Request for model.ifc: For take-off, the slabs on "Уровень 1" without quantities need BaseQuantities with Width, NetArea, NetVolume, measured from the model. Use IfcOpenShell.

First a look at what the model holds.

```python
import ifcopenshell
import ifcopenshell.util.element
import ifcopenshell.util.unit

model = ifcopenshell.open("model.ifc")
print(model.schema)
for unit_type in ("LENGTHUNIT", "AREAUNIT", "VOLUMEUNIT"):
    print(unit_type, ifcopenshell.util.unit.calculate_unit_scale(model, unit_type))
storey = next(s for s in model.by_type("IfcBuildingStorey") if s.Name == "Уровень 1")
slabs = [e for e in ifcopenshell.util.element.get_decomposition(storey) if e.is_a("IfcSlab")]
for e in sorted(slabs, key=lambda e: e.id()):
    print(e.id(), e.is_a(), e.Name, list(ifcopenshell.util.element.get_psets(e, qtos_only=True)), sep=" | ")
```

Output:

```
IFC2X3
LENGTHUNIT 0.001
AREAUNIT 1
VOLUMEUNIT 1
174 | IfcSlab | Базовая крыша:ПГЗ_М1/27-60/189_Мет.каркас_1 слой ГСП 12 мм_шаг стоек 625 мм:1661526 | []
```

```python
import ifcopenshell
import ifcopenshell.api.pset
import ifcopenshell.geom
import ifcopenshell.util.element
import ifcopenshell.util.shape
import ifcopenshell.util.unit

model = ifcopenshell.open("model.ifc")
unit_scale = ifcopenshell.util.unit.calculate_unit_scale(model)
area_scale = ifcopenshell.util.unit.calculate_unit_scale(model, "AREAUNIT")
volume_scale = ifcopenshell.util.unit.calculate_unit_scale(model, "VOLUMEUNIT")
settings = ifcopenshell.geom.settings()

storey = next(s for s in model.by_type("IfcBuildingStorey") if s.Name == "Уровень 1")
slabs = [e for e in ifcopenshell.util.element.get_decomposition(storey) if e.is_a("IfcSlab")]

for e in sorted(slabs, key=lambda e: e.id()):
    if ifcopenshell.util.element.get_psets(e, qtos_only=True, should_inherit=False):
        continue
    # Geometry comes back in metres, in the element's own axes.
    shape = ifcopenshell.geom.create_shape(settings, e)
    values = {
        "Width": ifcopenshell.util.shape.get_z(shape.geometry) / unit_scale,
        "NetArea": ifcopenshell.util.shape.get_footprint_area(shape.geometry) / area_scale,
        "NetVolume": ifcopenshell.util.shape.get_volume(shape.geometry) / volume_scale,
    }
    qto = ifcopenshell.api.pset.add_qto(model, product=e, name="BaseQuantities")
    ifcopenshell.api.pset.edit_qto(model, qto=qto, properties=values)
    print(e.id(), {k: round(v, 3) for k, v in values.items()})

model.write("model_v2.ifc")
```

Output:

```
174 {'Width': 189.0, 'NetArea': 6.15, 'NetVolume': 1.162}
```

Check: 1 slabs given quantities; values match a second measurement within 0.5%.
